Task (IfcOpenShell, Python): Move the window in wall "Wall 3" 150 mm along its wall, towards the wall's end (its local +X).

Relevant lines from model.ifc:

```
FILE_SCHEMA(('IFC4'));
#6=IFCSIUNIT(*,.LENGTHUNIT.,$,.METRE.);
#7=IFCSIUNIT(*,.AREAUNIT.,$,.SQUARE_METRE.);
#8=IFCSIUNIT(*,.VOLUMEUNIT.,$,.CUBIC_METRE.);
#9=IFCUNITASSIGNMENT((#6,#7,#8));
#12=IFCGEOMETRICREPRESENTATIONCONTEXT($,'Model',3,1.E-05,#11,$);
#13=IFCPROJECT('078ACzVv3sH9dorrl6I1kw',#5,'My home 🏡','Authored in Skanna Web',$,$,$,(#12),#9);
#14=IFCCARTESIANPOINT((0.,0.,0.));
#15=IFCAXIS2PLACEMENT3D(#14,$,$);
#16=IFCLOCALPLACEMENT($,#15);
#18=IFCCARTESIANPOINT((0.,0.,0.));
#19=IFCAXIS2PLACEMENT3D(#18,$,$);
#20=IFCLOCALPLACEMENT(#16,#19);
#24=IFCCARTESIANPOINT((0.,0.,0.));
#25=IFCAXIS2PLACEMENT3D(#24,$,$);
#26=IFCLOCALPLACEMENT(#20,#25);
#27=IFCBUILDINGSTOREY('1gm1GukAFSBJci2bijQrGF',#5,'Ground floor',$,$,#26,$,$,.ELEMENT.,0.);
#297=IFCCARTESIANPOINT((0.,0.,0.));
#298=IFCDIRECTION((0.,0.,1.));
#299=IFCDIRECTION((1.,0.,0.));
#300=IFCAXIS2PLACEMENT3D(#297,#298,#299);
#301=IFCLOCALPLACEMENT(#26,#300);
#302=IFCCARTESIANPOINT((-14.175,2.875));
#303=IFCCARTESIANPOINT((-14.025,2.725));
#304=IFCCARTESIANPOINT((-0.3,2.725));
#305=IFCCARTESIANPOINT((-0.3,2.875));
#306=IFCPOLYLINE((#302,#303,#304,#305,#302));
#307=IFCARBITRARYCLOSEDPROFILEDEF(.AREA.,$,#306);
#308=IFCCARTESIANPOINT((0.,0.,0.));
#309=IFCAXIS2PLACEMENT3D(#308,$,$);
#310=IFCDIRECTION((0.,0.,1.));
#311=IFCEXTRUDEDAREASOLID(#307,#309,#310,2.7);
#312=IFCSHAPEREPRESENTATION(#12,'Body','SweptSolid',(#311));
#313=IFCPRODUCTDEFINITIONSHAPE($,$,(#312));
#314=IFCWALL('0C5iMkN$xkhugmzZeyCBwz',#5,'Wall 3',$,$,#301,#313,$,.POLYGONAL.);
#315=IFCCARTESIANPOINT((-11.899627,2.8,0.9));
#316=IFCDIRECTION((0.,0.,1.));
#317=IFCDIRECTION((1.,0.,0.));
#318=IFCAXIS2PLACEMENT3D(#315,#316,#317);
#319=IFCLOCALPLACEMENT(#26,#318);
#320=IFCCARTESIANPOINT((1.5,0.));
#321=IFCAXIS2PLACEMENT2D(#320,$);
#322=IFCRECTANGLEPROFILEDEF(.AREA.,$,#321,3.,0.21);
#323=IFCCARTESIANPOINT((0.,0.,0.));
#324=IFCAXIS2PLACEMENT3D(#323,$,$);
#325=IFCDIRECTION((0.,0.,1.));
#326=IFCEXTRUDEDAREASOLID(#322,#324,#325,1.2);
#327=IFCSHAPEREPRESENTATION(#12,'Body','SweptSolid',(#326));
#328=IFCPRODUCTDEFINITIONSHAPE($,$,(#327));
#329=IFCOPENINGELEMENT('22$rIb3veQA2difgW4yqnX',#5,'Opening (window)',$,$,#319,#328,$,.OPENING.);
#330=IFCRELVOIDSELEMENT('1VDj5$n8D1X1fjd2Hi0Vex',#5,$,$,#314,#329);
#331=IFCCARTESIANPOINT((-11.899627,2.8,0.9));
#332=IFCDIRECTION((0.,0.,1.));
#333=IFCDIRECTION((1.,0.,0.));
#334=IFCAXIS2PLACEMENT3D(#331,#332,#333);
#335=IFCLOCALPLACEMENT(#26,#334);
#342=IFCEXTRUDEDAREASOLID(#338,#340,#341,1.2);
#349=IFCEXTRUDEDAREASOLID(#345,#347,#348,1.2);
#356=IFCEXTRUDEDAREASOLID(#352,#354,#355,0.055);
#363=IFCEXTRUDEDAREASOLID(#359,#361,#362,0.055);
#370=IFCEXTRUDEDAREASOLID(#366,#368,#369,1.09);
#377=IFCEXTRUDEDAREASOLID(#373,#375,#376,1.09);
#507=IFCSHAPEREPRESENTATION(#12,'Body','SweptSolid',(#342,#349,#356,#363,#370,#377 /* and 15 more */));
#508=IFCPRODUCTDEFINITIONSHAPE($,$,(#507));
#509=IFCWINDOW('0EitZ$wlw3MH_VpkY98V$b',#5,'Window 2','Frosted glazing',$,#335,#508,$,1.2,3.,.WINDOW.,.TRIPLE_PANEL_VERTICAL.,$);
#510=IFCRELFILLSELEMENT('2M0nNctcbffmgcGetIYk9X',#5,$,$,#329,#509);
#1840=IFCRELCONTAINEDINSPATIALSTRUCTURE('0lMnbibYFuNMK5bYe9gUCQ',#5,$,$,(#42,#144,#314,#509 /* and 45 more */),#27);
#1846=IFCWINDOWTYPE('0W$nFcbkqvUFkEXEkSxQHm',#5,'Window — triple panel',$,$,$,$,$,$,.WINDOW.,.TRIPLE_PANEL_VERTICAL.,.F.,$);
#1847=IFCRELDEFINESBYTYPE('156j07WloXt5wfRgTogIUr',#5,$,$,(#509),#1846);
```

```python
import ifcopenshell
import ifcopenshell.api.geometry
import ifcopenshell.util.placement
import ifcopenshell.util.unit

model = ifcopenshell.open("model.ifc")
unit_scale = ifcopenshell.util.unit.calculate_unit_scale(model)

window = model.by_guid("0EitZ$wlw3MH_VpkY98V$b")
opening = window.FillsVoids[0].RelatingOpeningElement
wall = opening.VoidsElements[0].RelatingBuildingElement

wall_matrix = ifcopenshell.util.placement.get_local_placement(wall.ObjectPlacement)
shift = wall_matrix[:3, 0] * 0.15 / unit_scale
before = ifcopenshell.util.placement.get_local_placement(window.ObjectPlacement)[:3, 3].copy()

# The window is not placed relative to its opening, so move both.
for product in (opening, window):
    matrix = ifcopenshell.util.placement.get_local_placement(product.ObjectPlacement)
    matrix[:3, 3] += shift
    ifcopenshell.api.geometry.edit_object_placement(model, product=product, matrix=matrix, is_si=False)

after = ifcopenshell.util.placement.get_local_placement(window.ObjectPlacement)[:3, 3]
print("window moved by", (after - before).round(3) + 0.0)

model.write("model-out.ifc")
```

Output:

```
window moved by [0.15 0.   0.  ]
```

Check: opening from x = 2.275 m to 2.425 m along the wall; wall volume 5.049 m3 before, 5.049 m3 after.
